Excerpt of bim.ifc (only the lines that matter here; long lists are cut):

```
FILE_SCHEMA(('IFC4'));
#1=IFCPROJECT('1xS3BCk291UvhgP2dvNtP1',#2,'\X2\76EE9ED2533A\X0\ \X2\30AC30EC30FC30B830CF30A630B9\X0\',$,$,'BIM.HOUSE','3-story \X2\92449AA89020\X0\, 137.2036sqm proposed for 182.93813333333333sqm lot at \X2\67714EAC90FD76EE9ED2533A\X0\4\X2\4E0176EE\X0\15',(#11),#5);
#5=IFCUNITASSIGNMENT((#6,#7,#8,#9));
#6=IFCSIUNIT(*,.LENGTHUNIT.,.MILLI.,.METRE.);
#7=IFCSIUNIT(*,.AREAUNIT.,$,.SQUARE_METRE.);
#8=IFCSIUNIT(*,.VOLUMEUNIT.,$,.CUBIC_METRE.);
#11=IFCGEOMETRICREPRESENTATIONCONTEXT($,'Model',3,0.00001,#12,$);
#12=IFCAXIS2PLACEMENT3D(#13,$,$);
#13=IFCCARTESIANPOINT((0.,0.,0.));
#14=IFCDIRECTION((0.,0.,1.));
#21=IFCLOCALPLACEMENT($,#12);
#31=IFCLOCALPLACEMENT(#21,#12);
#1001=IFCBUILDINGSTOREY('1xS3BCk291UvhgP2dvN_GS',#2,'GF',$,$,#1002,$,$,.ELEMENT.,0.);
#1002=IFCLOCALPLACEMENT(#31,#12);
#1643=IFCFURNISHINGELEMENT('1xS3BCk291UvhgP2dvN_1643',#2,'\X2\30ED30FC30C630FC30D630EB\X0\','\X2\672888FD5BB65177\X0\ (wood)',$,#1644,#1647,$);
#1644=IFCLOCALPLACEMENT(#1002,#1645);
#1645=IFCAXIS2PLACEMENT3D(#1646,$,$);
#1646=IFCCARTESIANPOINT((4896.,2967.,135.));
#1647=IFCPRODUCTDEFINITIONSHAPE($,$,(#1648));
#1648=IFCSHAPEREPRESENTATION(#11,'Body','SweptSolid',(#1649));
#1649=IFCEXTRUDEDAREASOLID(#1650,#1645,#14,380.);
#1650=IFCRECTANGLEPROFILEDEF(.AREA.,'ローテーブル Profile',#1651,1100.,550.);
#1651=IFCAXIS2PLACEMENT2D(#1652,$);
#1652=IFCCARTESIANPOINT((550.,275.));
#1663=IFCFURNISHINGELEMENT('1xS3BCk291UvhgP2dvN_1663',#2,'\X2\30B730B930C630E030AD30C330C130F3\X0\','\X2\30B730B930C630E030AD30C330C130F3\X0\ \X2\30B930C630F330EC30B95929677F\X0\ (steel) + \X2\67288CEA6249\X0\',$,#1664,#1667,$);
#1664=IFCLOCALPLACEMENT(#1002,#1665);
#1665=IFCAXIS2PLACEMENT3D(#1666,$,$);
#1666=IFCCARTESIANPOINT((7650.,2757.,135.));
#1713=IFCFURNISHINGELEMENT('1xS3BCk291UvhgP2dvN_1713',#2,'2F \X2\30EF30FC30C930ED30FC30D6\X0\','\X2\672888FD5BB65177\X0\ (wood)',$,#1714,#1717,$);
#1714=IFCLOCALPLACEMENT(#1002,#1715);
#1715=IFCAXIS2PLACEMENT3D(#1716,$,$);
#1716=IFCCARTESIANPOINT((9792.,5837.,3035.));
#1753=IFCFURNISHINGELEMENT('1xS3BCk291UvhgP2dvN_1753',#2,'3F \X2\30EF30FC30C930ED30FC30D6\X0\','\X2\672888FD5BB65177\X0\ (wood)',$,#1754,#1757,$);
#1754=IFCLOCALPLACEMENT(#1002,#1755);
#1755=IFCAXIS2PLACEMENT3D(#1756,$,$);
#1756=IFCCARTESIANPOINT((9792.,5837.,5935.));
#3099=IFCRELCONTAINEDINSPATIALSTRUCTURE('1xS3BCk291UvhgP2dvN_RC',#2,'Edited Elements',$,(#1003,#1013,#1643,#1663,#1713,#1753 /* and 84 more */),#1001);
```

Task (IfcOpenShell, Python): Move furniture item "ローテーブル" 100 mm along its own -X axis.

```python
import ifcopenshell
import ifcopenshell.api.geometry
import ifcopenshell.util.placement
import ifcopenshell.util.unit

model = ifcopenshell.open("bim.ifc")
unit_scale = ifcopenshell.util.unit.calculate_unit_scale(model)

item = model.by_id(1643)
matrix = ifcopenshell.util.placement.get_local_placement(item.ObjectPlacement)
matrix[:3, 3] -= matrix[:3, 0] * 0.1 / unit_scale
ifcopenshell.api.geometry.edit_object_placement(model, product=item, matrix=matrix, is_si=False)

print(ifcopenshell.util.placement.get_local_placement(item.ObjectPlacement).round(3) + 0.0)

model.write("bim_updated.ifc")
```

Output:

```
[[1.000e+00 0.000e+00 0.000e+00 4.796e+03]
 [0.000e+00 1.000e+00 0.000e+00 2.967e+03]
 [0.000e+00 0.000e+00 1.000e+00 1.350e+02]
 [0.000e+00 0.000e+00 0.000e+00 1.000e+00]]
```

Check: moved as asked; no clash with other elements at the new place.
